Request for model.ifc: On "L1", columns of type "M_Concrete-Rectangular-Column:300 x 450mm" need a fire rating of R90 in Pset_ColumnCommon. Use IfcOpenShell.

First a look at what the model holds.

```python
import ifcopenshell
import ifcopenshell.util.element

model = ifcopenshell.open("model.ifc")
print(model.schema)
storey = next(s for s in model.by_type("IfcBuildingStorey") if s.Name == "L1")
columns = [e for e in ifcopenshell.util.element.get_decomposition(storey) if e.is_a("IfcColumn")]
seen = {}
for e in columns:
    element_type = ifcopenshell.util.element.get_type(e)
    key = (element_type.Name if element_type != e and element_type else None, ifcopenshell.util.element.get_pset(e, "Pset_ColumnCommon", "FireRating"))
    seen[key] = seen.get(key, 0) + 1
for (name, value), count in sorted(seen.items(), key=str):
    print(count, "x", name, "|", value)
```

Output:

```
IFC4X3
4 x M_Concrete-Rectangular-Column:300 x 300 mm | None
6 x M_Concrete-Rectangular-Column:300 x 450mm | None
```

```python
import ifcopenshell
import ifcopenshell.api.pset
import ifcopenshell.util.element

model = ifcopenshell.open("model.ifc")

storey = next(s for s in model.by_type("IfcBuildingStorey") if s.Name == "L1")
columns = [e for e in ifcopenshell.util.element.get_decomposition(storey) if e.is_a("IfcColumn")]

count = 0
for e in columns:
    element_type = ifcopenshell.util.element.get_type(e)
    if element_type in (None, e) or element_type.Name != "M_Concrete-Rectangular-Column:300 x 450mm":
        continue
    # add_pset returns the element's existing set when there is one.
    pset = ifcopenshell.api.pset.add_pset(model, product=e, name="Pset_ColumnCommon")
    ifcopenshell.api.pset.edit_pset(model, pset=pset, properties={"FireRating": "R90"})
    count += 1

print(count, "columns updated")

model.write("model-out.ifc")
```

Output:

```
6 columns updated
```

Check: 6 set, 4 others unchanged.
